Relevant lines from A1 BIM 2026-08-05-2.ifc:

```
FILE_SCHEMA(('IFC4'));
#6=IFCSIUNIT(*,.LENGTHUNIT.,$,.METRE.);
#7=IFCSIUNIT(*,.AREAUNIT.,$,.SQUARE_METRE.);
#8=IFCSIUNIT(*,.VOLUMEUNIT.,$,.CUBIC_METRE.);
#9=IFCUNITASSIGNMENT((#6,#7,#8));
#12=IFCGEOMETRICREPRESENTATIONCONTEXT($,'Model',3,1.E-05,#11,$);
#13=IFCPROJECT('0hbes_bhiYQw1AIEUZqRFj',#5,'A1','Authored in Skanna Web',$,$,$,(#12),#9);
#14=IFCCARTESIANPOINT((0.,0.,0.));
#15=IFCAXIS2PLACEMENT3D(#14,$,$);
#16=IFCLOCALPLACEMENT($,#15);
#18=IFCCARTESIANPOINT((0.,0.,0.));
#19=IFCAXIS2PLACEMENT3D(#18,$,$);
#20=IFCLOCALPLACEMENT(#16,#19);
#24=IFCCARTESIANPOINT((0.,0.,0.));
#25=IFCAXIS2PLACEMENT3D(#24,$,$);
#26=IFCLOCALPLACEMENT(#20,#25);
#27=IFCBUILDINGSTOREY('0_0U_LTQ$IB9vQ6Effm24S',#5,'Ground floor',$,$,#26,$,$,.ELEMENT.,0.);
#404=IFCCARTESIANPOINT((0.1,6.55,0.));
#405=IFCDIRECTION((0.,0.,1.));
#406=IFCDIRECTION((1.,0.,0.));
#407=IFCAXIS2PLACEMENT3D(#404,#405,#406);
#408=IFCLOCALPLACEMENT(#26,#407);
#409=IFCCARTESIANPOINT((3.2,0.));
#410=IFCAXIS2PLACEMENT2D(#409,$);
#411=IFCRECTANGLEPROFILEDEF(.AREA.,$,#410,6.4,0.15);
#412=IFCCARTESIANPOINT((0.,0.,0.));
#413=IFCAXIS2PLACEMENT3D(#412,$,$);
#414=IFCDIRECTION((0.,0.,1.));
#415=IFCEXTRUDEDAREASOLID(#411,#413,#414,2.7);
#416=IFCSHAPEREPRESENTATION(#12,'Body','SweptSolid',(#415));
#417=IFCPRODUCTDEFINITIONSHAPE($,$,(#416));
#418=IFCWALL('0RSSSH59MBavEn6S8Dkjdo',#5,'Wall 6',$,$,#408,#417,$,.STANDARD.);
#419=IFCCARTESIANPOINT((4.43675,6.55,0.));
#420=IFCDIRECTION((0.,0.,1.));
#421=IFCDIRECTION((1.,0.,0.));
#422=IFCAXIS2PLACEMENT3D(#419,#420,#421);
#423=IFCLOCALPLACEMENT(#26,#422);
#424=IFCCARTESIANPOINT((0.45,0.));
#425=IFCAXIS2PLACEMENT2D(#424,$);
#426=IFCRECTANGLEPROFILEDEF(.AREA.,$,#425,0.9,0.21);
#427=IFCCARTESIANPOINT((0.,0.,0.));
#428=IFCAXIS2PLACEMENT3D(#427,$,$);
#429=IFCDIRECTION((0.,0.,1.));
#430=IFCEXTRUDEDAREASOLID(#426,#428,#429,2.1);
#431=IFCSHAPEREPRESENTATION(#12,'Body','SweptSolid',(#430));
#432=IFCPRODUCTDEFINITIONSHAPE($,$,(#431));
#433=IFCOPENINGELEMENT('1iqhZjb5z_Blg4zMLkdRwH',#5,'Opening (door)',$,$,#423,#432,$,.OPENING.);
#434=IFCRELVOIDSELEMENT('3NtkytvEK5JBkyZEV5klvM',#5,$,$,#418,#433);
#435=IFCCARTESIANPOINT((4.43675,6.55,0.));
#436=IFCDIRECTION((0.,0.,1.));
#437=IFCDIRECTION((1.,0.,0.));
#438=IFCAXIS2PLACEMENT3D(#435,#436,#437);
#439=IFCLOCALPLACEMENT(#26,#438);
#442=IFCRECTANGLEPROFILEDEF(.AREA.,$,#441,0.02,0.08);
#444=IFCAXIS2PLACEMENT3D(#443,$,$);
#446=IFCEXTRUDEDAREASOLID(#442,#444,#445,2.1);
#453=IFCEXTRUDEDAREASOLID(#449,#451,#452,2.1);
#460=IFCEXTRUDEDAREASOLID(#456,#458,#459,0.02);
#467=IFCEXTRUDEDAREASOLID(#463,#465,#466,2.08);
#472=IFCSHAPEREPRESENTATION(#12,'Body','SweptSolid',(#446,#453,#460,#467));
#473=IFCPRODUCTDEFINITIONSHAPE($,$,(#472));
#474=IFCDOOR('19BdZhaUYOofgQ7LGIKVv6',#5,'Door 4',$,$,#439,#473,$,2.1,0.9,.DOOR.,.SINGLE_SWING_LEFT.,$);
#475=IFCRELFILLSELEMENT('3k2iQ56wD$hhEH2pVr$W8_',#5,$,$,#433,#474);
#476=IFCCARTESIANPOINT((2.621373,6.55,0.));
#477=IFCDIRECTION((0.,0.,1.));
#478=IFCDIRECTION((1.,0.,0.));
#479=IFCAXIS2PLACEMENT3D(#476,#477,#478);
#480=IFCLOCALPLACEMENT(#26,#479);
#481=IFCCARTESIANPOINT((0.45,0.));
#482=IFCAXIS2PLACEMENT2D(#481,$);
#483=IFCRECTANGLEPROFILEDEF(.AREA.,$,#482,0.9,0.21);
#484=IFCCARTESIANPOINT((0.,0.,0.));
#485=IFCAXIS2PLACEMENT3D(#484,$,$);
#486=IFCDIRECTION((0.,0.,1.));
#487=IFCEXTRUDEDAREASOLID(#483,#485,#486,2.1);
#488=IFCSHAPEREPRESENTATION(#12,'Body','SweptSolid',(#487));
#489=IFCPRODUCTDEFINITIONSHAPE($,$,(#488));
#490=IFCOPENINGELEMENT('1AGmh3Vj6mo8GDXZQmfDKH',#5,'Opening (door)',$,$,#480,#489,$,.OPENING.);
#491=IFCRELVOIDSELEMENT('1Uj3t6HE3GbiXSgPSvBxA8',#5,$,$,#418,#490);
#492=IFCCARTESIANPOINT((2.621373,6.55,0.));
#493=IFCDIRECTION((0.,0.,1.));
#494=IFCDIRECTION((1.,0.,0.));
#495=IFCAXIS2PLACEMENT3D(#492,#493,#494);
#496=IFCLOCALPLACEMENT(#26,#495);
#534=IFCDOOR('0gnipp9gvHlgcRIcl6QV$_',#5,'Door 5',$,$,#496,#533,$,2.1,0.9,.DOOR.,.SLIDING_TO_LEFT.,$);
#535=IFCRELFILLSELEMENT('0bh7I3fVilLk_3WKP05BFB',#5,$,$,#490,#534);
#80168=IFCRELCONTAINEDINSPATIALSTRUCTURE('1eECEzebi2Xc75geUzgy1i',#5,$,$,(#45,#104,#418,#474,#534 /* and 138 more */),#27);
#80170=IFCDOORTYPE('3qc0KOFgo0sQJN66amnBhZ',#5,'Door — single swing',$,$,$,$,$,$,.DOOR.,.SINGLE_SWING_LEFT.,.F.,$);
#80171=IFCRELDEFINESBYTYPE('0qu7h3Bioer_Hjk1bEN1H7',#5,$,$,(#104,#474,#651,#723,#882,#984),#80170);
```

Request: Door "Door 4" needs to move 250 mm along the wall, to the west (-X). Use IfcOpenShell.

```python
import ifcopenshell
import ifcopenshell.api.geometry
import ifcopenshell.util.placement
import ifcopenshell.util.unit

model = ifcopenshell.open("A1 BIM 2026-08-05-2.ifc")
unit_scale = ifcopenshell.util.unit.calculate_unit_scale(model)

door = model.by_guid("19BdZhaUYOofgQ7LGIKVv6")
opening = door.FillsVoids[0].RelatingOpeningElement
wall = opening.VoidsElements[0].RelatingBuildingElement

wall_matrix = ifcopenshell.util.placement.get_local_placement(wall.ObjectPlacement)
shift = wall_matrix[:3, 0] * -0.25 / unit_scale
before = ifcopenshell.util.placement.get_local_placement(door.ObjectPlacement)[:3, 3].copy()

# The door is not placed relative to its opening, so move both.
for product in (opening, door):
    matrix = ifcopenshell.util.placement.get_local_placement(product.ObjectPlacement)
    matrix[:3, 3] += shift
    ifcopenshell.api.geometry.edit_object_placement(model, product=product, matrix=matrix, is_si=False)

after = ifcopenshell.util.placement.get_local_placement(door.ObjectPlacement)[:3, 3]
print("door moved by", (after - before).round(3) + 0.0)

model.write("A1 BIM 2026-08-05-2_updated.ifc")
```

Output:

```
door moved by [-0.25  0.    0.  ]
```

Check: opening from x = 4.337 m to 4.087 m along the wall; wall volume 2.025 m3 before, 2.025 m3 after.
